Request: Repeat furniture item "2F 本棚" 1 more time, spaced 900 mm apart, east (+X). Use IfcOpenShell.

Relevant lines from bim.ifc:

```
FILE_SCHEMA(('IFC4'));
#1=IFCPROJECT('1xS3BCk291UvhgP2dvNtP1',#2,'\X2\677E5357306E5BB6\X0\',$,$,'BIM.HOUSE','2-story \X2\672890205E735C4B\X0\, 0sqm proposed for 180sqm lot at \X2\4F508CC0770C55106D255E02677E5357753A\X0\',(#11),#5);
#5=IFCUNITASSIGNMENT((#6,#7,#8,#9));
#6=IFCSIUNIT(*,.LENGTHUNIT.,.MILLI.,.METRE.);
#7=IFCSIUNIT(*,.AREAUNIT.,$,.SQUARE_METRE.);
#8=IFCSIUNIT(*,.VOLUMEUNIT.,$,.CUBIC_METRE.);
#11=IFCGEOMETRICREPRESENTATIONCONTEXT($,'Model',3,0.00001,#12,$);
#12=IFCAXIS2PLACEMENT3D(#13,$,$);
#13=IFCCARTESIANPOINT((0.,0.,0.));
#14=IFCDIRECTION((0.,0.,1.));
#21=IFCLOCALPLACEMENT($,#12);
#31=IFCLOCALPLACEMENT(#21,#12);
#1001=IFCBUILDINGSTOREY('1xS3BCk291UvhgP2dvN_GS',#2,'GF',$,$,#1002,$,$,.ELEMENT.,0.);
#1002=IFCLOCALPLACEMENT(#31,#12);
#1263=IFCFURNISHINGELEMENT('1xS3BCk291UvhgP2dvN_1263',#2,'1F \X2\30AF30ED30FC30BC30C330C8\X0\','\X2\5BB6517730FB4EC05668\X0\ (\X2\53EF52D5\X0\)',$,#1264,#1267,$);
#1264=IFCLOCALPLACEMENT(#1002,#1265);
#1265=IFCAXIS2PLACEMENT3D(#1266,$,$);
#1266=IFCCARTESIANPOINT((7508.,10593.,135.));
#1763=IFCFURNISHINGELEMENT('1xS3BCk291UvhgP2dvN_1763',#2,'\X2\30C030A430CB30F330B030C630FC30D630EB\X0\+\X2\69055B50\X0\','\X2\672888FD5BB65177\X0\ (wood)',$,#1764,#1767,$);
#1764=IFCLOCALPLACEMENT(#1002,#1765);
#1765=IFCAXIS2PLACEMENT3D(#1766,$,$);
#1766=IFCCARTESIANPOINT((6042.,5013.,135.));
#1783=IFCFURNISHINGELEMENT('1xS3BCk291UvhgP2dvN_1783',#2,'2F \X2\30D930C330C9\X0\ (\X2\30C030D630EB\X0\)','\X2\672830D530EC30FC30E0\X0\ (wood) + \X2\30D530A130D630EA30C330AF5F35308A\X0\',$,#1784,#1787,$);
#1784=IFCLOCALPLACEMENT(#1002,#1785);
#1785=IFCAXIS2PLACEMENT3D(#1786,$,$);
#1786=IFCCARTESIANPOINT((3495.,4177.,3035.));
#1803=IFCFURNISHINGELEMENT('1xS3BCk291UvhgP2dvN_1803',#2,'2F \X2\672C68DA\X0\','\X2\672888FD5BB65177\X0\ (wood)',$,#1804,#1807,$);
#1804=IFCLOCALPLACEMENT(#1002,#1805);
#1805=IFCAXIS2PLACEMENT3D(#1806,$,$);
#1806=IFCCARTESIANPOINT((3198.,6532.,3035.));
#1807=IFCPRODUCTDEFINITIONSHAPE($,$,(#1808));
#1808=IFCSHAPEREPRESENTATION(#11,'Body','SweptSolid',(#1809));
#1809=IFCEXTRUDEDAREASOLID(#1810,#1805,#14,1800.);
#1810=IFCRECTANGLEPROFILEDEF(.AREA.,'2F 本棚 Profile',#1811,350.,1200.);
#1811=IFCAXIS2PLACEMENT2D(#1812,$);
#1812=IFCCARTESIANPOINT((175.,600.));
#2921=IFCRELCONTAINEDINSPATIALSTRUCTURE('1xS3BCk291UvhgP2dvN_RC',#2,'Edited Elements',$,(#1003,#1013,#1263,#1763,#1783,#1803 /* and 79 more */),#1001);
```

```python
import numpy as np
import ifcopenshell
import ifcopenshell.api.geometry
import ifcopenshell.api.root
import ifcopenshell.util.element
import ifcopenshell.util.placement
import ifcopenshell.util.unit

model = ifcopenshell.open("bim.ifc")
unit_scale = ifcopenshell.util.unit.calculate_unit_scale(model)


def reuse_history(source, copy):
    """copy_class also copies each property set's owner history, people and application; keep the originals."""
    for rel in copy.IsDefinedBy:
        if rel.is_a("IfcRelDefinesByProperties") and (history := rel.RelatingPropertyDefinition.OwnerHistory):
            rel.RelatingPropertyDefinition.OwnerHistory = source.OwnerHistory
            ifcopenshell.util.element.remove_deep2(model, history)


source = model.by_id(1803)
base = ifcopenshell.util.placement.get_local_placement(source.ObjectPlacement)
step = np.array([1.0, 0.0, 0.0]) * 0.9 / unit_scale

for i in range(1, 2):
    copy = ifcopenshell.api.root.copy_class(model, product=source)
    copy.Representation = ifcopenshell.util.element.copy_deep(
        model, source.Representation, exclude=["IfcGeometricRepresentationContext", "IfcRepresentationMap"]
    )
    reuse_history(source, copy)
    matrix = base.copy()
    matrix[:3, 3] += i * step
    print("added at", matrix[:3, 3].round(3) + 0.0)
    ifcopenshell.api.geometry.edit_object_placement(model, product=copy, matrix=matrix, is_si=False)

model.write("bim-out.ifc")
```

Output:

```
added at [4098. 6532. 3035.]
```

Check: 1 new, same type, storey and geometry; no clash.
